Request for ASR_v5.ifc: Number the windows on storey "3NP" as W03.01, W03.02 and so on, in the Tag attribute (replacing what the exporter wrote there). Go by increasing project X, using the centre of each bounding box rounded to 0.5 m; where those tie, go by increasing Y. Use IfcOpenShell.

First a look at what the model holds.

```python
import ifcopenshell
import ifcopenshell.util.element
import ifcopenshell.util.placement

model = ifcopenshell.open("ASR_v5.ifc")
print(model.schema)
storey = next(s for s in model.by_type("IfcBuildingStorey") if s.Name == "3NP")
windows = [e for e in ifcopenshell.util.element.get_decomposition(storey) if e.is_a("IfcWindow")]
for e in sorted(windows, key=lambda e: e.id()):
    origin = ifcopenshell.util.placement.get_local_placement(e.ObjectPlacement)[:3, 3]
    print(e.id(), e.Tag, e.Name, origin.round(2) + 0.0, sep=" | ")
```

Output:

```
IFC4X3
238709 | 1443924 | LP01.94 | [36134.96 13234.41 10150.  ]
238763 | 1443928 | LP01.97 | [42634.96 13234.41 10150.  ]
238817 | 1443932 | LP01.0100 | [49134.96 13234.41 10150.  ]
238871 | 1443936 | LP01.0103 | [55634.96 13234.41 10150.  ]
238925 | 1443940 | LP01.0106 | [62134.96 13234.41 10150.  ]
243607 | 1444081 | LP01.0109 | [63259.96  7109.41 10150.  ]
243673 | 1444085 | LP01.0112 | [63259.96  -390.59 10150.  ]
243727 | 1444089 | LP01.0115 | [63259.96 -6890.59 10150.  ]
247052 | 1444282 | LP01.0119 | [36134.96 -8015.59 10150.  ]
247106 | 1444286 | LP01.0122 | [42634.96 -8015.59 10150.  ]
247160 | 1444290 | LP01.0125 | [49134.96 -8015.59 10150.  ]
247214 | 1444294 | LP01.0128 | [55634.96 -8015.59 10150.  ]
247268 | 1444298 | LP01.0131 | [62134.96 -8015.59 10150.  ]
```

```python
import ifcopenshell
import ifcopenshell.geom
import ifcopenshell.util.element
import ifcopenshell.util.shape

model = ifcopenshell.open("ASR_v5.ifc")
settings = ifcopenshell.geom.settings()
settings.set("use-world-coords", True)


def centre(element):
    shape = ifcopenshell.geom.create_shape(settings, element)
    return ifcopenshell.util.shape.get_bbox_centroid(shape.geometry)


storey = next(s for s in model.by_type("IfcBuildingStorey") if s.Name == "3NP")
windows = [e for e in ifcopenshell.util.element.get_decomposition(storey) if e.is_a("IfcWindow")]

# Insertion points can sit at a corner or the storey origin, so sort by the geometry (in metres).
centres = {e: centre(e) for e in windows}
windows.sort(key=lambda e: (round(centres[e][0] / 0.5), centres[e][1]))

for i, e in enumerate(windows, start=1):
    number = f"W03.{i:02d}"
    e.Tag = number
    print(e.id(), number)

model.write("ASR_v5_updated.ifc")
```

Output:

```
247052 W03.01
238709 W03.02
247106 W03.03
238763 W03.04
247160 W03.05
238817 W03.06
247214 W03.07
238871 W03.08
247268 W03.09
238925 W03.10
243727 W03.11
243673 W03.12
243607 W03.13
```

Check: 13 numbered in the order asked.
